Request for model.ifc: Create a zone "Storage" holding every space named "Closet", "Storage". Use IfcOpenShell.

First a look at what the model holds.

```python
import ifcopenshell

model = ifcopenshell.open("model.ifc")
print(model.schema)
seen = {}
for space in model.by_type("IfcSpace"):
    seen[space.LongName] = seen.get(space.LongName, 0) + 1
for name, count in sorted(seen.items(), key=str):
    print(count, "x", name)
print("zones:", [z.Name for z in model.by_type("IfcZone")][:20])
```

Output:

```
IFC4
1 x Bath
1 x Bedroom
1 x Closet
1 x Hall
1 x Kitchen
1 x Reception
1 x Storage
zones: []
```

```python
import ifcopenshell
import ifcopenshell.api.group
import ifcopenshell.api.root

model = ifcopenshell.open("model.ifc")

names = {"Closet", "Storage"}
spaces = [s for s in model.by_type("IfcSpace") if s.LongName in names]

zone = ifcopenshell.api.root.create_entity(model, ifc_class="IfcZone", name="Storage")
ifcopenshell.api.group.assign_group(model, products=spaces, group=zone)
print(len(spaces), "spaces in", zone.Name)

model.write("model_rev.ifc")
```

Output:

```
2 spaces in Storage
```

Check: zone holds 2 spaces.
